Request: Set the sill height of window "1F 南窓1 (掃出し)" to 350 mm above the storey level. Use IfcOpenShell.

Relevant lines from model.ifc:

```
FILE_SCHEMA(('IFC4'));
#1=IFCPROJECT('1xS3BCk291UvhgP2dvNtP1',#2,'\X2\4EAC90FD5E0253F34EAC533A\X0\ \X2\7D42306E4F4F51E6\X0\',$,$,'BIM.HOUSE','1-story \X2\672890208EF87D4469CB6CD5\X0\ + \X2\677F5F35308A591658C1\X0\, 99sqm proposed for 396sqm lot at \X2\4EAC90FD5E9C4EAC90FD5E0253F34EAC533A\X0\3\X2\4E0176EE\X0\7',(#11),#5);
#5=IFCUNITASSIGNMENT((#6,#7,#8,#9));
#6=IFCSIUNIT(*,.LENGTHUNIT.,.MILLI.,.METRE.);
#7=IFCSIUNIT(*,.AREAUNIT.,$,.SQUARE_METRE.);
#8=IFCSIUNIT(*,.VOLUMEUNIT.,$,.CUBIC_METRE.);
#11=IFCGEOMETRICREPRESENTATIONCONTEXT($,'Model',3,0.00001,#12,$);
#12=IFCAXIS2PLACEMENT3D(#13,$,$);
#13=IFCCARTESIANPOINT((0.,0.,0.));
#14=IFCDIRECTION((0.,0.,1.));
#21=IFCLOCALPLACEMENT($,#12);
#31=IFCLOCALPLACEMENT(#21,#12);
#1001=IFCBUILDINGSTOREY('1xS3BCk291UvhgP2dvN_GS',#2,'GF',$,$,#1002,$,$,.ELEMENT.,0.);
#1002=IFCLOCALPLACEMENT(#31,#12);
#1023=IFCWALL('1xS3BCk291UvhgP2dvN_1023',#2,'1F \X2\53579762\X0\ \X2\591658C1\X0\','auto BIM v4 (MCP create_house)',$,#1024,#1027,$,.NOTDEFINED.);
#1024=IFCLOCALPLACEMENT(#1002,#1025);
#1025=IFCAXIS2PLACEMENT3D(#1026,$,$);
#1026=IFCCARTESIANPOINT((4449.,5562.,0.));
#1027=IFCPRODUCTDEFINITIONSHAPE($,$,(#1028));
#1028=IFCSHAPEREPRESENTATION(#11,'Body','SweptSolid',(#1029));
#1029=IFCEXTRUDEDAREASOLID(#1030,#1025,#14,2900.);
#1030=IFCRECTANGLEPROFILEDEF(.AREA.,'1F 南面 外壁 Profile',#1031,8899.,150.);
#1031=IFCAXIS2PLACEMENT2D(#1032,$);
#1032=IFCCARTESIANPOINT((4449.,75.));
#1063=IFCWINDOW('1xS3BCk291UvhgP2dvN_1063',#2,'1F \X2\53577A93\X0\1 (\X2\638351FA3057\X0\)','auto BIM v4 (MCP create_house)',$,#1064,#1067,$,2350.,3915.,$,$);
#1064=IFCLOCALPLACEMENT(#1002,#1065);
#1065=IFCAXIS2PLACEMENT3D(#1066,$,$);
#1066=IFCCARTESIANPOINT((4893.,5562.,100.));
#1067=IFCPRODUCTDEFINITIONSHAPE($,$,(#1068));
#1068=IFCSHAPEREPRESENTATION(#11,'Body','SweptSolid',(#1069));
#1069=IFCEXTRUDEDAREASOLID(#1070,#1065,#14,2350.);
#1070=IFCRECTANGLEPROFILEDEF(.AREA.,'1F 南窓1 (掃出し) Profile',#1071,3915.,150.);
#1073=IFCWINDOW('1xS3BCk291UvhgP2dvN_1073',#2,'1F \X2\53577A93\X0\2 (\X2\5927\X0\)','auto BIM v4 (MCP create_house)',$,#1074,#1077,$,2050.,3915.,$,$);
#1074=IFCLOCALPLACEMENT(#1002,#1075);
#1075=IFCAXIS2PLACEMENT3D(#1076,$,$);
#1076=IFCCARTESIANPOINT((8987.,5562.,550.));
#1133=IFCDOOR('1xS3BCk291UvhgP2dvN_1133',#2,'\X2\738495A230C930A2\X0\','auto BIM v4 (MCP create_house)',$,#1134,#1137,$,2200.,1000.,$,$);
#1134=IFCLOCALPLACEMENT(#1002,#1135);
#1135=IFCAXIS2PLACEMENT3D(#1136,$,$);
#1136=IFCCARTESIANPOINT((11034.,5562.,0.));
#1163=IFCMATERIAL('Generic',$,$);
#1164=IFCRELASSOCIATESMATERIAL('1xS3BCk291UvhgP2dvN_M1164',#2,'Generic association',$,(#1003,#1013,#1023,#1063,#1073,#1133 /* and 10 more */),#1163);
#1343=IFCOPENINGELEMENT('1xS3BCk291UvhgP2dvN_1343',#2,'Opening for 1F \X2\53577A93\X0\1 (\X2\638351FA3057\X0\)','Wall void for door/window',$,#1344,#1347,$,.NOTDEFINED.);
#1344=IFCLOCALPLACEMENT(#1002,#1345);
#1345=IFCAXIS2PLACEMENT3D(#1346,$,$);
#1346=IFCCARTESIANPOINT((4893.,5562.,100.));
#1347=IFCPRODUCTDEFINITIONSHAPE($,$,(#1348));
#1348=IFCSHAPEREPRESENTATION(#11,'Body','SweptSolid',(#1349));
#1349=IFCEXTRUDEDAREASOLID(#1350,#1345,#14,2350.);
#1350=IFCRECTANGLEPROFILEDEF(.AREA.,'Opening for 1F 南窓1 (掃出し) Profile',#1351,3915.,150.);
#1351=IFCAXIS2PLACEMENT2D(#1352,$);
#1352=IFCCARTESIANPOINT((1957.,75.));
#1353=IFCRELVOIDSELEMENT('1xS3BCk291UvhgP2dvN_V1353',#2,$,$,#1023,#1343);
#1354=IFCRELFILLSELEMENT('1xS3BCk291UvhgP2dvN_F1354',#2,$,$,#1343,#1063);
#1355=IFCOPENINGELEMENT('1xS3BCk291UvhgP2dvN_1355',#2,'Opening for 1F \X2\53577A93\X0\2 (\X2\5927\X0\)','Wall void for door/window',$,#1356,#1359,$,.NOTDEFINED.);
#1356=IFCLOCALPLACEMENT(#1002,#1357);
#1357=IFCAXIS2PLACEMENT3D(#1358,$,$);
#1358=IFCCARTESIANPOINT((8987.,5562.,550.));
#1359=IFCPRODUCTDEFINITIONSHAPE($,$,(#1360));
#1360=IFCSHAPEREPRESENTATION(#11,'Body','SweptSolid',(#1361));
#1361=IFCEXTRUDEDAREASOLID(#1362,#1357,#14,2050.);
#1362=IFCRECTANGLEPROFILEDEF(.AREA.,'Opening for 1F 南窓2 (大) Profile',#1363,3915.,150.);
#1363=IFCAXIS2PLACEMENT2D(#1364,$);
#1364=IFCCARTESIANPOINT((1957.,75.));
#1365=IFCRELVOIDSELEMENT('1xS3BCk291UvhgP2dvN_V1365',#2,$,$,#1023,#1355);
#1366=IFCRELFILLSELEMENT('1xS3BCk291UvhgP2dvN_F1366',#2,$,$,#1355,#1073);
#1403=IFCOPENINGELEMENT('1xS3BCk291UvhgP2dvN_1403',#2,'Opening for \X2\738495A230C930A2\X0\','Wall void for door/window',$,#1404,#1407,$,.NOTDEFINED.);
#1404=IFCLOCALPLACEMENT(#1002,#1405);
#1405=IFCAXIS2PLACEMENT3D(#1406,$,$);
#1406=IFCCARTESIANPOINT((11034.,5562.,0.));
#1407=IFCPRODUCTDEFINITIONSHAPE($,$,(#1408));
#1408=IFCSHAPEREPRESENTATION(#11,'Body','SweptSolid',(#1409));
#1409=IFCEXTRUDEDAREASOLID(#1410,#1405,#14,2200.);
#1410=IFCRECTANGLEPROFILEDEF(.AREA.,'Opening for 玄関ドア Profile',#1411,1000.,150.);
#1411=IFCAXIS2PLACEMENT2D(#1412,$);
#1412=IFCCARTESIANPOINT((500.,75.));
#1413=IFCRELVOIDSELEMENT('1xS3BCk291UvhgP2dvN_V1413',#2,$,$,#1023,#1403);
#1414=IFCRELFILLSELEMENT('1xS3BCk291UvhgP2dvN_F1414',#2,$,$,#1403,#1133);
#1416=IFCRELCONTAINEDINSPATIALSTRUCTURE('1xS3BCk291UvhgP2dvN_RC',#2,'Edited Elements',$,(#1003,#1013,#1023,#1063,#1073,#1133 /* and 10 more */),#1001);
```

```python
import numpy as np
import ifcopenshell
import ifcopenshell.api.geometry
import ifcopenshell.geom
import ifcopenshell.util.element
import ifcopenshell.util.placement
import ifcopenshell.util.shape
import ifcopenshell.util.unit

model = ifcopenshell.open("model.ifc")
unit_scale = ifcopenshell.util.unit.calculate_unit_scale(model)

window = model.by_guid("1xS3BCk291UvhgP2dvN_1063")
opening = window.FillsVoids[0].RelatingOpeningElement
storey = ifcopenshell.util.element.get_container(window, ifc_class="IfcBuildingStorey")
level = ifcopenshell.util.placement.get_local_placement(storey.ObjectPlacement)[2, 3]

# The opening's origin need not be at the sill, so measure its lowest point.
shape = ifcopenshell.geom.create_shape(ifcopenshell.geom.settings(), opening)
bottom = ifcopenshell.util.shape.get_shape_bottom_elevation(shape, shape.geometry) / unit_scale
dz = level + 0.35 / unit_scale - bottom

shift = np.array([0.0, 0.0, dz])
# The window is not placed relative to its opening, so move both.
for product in (opening, window):
    matrix = ifcopenshell.util.placement.get_local_placement(product.ObjectPlacement)
    matrix[:3, 3] += shift
    ifcopenshell.api.geometry.edit_object_placement(model, product=product, matrix=matrix, is_si=False)

print(f"moved by {dz * unit_scale:+.3f} m")

model.write("model-out.ifc")
```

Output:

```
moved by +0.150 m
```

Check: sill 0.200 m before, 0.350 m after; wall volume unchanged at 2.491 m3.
